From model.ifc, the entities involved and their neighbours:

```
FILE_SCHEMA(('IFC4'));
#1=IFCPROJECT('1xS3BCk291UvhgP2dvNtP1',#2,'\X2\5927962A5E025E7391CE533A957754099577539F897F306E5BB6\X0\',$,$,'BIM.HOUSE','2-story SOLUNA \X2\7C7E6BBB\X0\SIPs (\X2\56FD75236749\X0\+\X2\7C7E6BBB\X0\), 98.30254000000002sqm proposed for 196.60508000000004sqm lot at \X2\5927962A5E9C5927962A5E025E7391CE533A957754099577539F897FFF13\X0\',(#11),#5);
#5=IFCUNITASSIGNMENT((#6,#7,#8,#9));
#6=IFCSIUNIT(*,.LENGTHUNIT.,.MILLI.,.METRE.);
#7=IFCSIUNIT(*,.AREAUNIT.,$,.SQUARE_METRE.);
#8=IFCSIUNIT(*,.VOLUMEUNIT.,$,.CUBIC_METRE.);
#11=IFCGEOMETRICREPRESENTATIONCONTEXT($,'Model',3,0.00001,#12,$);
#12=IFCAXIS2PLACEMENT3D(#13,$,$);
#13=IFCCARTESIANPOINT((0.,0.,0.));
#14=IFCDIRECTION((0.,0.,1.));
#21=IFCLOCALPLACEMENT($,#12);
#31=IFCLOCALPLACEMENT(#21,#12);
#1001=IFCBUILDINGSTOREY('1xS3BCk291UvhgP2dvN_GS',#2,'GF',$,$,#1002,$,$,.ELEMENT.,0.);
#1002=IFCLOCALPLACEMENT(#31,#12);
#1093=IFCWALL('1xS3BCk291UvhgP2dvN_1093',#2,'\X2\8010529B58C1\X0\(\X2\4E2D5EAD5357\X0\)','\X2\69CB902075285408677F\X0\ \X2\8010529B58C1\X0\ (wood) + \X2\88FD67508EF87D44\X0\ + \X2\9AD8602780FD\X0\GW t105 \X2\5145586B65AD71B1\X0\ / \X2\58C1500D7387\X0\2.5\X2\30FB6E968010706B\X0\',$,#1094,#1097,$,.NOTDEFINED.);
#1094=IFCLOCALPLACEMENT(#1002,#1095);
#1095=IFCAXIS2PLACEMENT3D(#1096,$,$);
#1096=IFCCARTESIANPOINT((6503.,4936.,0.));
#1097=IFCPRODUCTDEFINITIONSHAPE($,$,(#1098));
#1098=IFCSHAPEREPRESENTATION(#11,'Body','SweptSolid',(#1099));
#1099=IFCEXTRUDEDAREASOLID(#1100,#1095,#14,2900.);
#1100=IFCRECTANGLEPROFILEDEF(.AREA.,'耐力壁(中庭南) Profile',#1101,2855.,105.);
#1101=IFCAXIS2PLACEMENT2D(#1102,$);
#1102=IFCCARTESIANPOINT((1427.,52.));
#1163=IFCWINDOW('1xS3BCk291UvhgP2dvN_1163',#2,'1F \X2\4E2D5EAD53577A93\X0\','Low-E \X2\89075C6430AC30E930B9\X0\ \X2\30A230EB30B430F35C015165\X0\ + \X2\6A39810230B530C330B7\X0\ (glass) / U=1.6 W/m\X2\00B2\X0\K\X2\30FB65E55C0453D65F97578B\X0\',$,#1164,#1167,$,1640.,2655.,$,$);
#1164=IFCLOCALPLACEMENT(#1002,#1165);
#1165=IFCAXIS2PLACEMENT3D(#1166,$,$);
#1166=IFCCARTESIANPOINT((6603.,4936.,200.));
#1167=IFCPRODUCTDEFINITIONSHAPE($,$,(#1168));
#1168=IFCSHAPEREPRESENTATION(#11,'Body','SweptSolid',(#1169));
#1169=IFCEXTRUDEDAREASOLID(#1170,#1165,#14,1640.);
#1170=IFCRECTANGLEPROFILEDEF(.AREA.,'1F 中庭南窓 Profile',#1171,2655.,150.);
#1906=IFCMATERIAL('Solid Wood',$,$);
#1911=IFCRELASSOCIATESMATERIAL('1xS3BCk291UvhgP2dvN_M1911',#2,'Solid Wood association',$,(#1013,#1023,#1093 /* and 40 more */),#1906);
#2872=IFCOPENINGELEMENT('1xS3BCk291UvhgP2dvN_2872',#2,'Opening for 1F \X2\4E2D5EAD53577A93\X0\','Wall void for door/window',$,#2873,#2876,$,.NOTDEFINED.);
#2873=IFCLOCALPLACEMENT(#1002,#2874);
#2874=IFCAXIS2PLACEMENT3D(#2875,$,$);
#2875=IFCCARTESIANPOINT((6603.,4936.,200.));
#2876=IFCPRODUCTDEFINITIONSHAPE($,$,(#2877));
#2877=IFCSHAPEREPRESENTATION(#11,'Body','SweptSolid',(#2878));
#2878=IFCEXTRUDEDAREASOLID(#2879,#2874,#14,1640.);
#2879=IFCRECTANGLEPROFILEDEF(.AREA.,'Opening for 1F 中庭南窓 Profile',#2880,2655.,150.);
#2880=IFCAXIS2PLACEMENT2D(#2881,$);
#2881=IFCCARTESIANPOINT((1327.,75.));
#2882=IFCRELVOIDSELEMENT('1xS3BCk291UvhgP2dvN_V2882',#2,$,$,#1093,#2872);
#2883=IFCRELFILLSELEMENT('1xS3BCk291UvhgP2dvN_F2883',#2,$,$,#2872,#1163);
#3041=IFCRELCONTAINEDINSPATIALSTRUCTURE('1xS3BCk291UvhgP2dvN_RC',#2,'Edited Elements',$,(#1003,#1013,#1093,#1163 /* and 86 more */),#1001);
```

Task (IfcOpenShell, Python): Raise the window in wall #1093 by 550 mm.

```python
import numpy as np
import ifcopenshell
import ifcopenshell.api.geometry
import ifcopenshell.util.placement
import ifcopenshell.util.unit

model = ifcopenshell.open("model.ifc")
unit_scale = ifcopenshell.util.unit.calculate_unit_scale(model)

window = model.by_guid("1xS3BCk291UvhgP2dvN_1163")
opening = window.FillsVoids[0].RelatingOpeningElement
dz = 0.55 / unit_scale

shift = np.array([0.0, 0.0, dz])
# The window is not placed relative to its opening, so move both.
for product in (opening, window):
    matrix = ifcopenshell.util.placement.get_local_placement(product.ObjectPlacement)
    matrix[:3, 3] += shift
    ifcopenshell.api.geometry.edit_object_placement(model, product=product, matrix=matrix, is_si=False)

print(f"moved by {dz * unit_scale:+.3f} m")

model.write("model_updated.ifc")
```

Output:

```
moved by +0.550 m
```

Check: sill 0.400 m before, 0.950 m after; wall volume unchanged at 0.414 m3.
